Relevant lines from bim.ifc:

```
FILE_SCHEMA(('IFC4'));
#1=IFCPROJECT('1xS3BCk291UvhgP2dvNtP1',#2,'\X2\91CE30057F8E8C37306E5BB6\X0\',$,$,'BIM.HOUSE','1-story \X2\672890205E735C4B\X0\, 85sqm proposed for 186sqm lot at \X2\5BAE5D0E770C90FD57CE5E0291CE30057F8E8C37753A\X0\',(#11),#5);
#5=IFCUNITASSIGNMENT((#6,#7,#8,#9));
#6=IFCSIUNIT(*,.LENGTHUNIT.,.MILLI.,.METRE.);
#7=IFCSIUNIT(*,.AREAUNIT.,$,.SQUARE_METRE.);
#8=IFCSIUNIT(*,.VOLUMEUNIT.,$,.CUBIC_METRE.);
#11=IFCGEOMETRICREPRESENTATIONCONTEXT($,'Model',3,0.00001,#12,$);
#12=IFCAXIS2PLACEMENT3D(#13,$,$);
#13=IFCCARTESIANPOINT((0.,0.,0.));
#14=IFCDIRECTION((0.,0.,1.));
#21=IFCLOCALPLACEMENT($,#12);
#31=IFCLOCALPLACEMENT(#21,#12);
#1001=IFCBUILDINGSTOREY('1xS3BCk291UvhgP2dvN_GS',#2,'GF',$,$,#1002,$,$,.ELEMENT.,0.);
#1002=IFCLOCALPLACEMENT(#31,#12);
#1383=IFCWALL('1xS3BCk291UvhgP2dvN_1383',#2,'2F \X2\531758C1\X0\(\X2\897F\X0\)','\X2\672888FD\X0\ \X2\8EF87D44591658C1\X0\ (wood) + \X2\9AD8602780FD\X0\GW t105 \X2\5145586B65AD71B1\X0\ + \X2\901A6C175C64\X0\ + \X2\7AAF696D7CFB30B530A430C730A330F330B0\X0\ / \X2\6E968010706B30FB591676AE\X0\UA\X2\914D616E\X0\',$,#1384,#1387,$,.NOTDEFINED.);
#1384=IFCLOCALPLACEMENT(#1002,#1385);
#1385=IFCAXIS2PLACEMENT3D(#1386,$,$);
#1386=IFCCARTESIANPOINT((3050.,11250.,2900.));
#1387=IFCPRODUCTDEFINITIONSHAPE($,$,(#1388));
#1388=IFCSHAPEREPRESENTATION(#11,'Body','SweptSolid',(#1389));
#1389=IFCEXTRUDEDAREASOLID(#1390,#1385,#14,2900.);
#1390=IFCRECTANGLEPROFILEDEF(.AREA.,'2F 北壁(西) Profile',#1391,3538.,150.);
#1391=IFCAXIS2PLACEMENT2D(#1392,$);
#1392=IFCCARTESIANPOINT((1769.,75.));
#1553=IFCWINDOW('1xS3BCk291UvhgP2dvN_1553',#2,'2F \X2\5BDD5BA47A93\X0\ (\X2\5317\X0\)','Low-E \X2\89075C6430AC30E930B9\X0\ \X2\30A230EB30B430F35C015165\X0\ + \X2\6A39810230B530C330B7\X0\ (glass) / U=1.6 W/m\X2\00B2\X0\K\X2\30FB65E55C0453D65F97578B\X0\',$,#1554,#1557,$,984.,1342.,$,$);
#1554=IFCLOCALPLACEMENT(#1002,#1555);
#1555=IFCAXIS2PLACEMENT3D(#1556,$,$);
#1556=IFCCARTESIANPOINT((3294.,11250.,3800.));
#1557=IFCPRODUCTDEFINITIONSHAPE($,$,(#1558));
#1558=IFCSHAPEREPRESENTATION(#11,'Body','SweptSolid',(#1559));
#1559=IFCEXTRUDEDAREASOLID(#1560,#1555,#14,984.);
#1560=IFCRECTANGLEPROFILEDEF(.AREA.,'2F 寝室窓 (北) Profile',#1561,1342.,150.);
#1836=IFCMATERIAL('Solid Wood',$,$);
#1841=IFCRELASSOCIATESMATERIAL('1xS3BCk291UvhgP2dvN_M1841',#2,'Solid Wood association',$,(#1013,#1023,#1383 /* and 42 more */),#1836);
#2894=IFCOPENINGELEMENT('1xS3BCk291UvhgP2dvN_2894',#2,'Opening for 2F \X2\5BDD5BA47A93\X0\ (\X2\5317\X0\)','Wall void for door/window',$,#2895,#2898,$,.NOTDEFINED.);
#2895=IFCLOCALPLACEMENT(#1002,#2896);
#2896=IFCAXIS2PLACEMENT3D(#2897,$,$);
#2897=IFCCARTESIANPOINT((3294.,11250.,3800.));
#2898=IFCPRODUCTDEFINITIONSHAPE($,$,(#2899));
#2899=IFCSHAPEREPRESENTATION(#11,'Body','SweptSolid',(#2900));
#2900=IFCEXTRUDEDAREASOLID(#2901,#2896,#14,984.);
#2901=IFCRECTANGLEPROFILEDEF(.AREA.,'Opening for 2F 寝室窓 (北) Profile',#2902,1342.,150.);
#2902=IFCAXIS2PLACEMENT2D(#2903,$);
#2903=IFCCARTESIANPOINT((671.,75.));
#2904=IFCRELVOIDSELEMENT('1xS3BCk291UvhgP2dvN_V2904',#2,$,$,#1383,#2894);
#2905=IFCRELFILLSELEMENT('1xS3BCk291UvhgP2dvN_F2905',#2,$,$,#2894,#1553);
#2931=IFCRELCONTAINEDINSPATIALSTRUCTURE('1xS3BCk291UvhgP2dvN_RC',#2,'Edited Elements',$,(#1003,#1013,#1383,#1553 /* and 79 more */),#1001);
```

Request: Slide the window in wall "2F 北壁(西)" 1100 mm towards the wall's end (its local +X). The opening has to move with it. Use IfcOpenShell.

```python
import ifcopenshell
import ifcopenshell.api.geometry
import ifcopenshell.util.placement

model = ifcopenshell.open("bim.ifc")

window = model.by_guid("1xS3BCk291UvhgP2dvN_1553")
opening = window.FillsVoids[0].RelatingOpeningElement
wall = opening.VoidsElements[0].RelatingBuildingElement

wall_matrix = ifcopenshell.util.placement.get_local_placement(wall.ObjectPlacement)
shift = wall_matrix[:3, 0] * 1100.0
before = ifcopenshell.util.placement.get_local_placement(window.ObjectPlacement)[:3, 3].copy()

# The window is not placed relative to its opening, so move both.
for product in (opening, window):
    matrix = ifcopenshell.util.placement.get_local_placement(product.ObjectPlacement)
    matrix[:3, 3] += shift
    ifcopenshell.api.geometry.edit_object_placement(model, product=product, matrix=matrix, is_si=False)

after = ifcopenshell.util.placement.get_local_placement(window.ObjectPlacement)[:3, 3]
print("window moved by", (after - before).round(3) + 0.0)

model.write("bim_v2.ifc")
```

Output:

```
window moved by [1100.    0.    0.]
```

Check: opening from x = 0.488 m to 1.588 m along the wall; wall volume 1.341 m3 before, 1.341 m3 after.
